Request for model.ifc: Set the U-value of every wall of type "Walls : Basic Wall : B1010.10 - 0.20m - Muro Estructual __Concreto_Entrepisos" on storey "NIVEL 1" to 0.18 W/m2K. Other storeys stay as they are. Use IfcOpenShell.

First a look at what the model holds.

```python
import ifcopenshell
import ifcopenshell.util.element

model = ifcopenshell.open("model.ifc")
print(model.schema)
storey = next(s for s in model.by_type("IfcBuildingStorey") if s.Name == "NIVEL 1")
walls = [e for e in ifcopenshell.util.element.get_decomposition(storey) if e.is_a("IfcWall")]
seen = {}
for e in walls:
    element_type = ifcopenshell.util.element.get_type(e)
    key = (element_type.Name if element_type != e and element_type else None, ifcopenshell.util.element.get_pset(e, "Pset_WallCommon", "ThermalTransmittance"))
    seen[key] = seen.get(key, 0) + 1
for (name, value), count in sorted(seen.items(), key=str):
    print(count, "x", name, "|", value)
```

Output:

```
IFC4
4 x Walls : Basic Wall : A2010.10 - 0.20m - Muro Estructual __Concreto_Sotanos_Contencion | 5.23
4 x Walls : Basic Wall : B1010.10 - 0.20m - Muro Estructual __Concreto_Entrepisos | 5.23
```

```python
import ifcopenshell
import ifcopenshell.api.pset
import ifcopenshell.util.element

model = ifcopenshell.open("model.ifc")

storey = next(s for s in model.by_type("IfcBuildingStorey") if s.Name == "NIVEL 1")
walls = [e for e in ifcopenshell.util.element.get_decomposition(storey) if e.is_a("IfcWall")]

count = 0
for e in walls:
    element_type = ifcopenshell.util.element.get_type(e)
    if element_type in (None, e) or element_type.Name != "Walls : Basic Wall : B1010.10 - 0.20m - Muro Estructual __Concreto_Entrepisos":
        continue
    # add_pset returns the element's existing set when there is one.
    pset = ifcopenshell.api.pset.add_pset(model, product=e, name="Pset_WallCommon")
    ifcopenshell.api.pset.edit_pset(model, pset=pset, properties={"ThermalTransmittance": 0.18})
    count += 1

print(count, "walls updated")

model.write("model_v2.ifc")
```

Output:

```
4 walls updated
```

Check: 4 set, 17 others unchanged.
